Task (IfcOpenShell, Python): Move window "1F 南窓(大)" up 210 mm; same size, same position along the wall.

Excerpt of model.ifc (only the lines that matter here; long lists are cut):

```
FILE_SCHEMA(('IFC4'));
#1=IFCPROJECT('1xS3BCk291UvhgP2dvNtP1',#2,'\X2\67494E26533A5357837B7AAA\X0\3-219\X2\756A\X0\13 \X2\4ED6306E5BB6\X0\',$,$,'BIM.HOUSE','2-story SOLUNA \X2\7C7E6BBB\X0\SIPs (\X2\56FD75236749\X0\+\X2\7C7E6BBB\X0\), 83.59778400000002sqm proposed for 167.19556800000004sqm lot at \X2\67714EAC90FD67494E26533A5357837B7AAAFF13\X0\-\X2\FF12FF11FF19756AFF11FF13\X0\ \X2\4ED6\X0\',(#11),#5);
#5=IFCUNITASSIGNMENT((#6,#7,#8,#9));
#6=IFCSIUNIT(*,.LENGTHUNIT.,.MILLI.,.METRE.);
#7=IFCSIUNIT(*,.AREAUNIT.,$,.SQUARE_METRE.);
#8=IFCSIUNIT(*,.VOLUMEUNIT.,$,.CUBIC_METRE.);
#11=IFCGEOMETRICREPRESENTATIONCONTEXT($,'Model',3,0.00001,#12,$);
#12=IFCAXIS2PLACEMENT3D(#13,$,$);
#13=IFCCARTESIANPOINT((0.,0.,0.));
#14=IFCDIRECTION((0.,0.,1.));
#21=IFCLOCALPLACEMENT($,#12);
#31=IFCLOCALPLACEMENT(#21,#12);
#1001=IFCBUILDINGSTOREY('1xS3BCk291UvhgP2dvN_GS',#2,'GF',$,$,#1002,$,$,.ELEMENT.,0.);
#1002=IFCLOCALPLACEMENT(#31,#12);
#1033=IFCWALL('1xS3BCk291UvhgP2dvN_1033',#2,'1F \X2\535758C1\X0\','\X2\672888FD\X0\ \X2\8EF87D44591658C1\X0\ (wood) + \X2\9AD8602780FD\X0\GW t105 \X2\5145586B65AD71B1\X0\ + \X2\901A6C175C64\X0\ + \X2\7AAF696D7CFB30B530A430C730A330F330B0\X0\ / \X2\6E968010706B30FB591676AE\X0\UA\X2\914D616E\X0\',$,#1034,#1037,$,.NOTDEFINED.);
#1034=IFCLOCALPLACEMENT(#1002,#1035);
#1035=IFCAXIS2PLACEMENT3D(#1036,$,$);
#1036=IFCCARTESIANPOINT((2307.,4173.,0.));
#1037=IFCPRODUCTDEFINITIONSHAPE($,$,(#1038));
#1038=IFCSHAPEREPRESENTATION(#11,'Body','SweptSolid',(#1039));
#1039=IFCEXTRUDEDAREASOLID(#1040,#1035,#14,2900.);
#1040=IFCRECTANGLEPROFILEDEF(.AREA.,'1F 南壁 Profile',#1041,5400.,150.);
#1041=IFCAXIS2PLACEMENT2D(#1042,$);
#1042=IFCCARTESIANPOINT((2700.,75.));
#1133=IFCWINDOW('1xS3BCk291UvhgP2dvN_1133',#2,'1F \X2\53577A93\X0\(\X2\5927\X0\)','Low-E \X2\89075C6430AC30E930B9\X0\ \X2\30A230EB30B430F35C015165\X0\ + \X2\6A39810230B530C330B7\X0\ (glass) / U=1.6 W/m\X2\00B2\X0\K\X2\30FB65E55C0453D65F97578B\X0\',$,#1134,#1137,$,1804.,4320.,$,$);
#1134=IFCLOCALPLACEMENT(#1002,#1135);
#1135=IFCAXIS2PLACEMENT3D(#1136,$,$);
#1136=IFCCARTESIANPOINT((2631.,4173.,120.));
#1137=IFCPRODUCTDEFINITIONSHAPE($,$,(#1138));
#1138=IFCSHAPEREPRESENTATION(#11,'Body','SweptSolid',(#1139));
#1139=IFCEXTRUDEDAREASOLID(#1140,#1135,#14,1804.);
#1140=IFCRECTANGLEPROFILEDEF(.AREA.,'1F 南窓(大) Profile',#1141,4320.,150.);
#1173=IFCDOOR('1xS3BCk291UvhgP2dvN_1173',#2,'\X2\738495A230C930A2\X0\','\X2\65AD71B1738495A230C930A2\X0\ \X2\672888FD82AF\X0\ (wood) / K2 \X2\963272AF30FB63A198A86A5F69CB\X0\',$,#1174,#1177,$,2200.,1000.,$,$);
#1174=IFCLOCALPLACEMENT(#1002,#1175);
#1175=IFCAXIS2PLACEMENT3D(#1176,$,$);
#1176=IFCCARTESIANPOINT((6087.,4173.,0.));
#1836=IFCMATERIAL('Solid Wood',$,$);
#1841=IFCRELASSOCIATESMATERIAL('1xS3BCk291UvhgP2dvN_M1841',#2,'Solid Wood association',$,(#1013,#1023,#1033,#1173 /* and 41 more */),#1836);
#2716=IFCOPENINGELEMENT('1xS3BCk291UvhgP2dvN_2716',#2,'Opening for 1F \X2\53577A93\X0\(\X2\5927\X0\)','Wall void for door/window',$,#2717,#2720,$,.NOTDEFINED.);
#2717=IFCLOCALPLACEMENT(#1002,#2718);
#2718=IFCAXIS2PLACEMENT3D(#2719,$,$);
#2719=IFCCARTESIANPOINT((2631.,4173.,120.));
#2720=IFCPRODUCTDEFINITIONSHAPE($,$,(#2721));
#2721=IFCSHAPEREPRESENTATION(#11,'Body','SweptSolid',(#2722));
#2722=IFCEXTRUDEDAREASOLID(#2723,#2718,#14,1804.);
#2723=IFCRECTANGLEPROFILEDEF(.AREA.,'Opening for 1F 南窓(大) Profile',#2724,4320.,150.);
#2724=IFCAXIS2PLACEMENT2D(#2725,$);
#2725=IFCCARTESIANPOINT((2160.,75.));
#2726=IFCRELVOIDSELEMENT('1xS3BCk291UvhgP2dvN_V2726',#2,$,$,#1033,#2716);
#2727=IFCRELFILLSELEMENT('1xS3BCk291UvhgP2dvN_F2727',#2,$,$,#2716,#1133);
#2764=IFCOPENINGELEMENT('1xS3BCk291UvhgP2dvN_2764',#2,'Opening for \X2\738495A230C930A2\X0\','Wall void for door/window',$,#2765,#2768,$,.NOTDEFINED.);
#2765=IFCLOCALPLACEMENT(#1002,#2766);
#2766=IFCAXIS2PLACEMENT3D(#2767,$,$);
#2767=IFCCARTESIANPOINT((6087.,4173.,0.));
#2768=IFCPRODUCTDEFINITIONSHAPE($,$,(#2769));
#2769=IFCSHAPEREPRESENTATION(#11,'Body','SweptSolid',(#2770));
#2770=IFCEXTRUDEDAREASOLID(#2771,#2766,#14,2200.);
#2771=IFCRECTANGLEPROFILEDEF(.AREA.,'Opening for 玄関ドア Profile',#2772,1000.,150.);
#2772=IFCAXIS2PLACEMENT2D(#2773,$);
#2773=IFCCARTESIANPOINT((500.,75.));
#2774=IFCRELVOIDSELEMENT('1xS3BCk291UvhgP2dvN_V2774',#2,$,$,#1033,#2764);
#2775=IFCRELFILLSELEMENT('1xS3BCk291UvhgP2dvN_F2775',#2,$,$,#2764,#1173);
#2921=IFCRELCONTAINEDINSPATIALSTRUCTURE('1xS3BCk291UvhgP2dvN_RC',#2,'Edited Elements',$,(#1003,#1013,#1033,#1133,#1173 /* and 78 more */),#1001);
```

```python
import numpy as np
import ifcopenshell
import ifcopenshell.api.geometry
import ifcopenshell.util.placement
import ifcopenshell.util.unit

model = ifcopenshell.open("model.ifc")
unit_scale = ifcopenshell.util.unit.calculate_unit_scale(model)

window = model.by_guid("1xS3BCk291UvhgP2dvN_1133")
opening = window.FillsVoids[0].RelatingOpeningElement
dz = 210.0

shift = np.array([0.0, 0.0, dz])
# The window is not placed relative to its opening, so move both.
for product in (opening, window):
    matrix = ifcopenshell.util.placement.get_local_placement(product.ObjectPlacement)
    matrix[:3, 3] += shift
    ifcopenshell.api.geometry.edit_object_placement(model, product=product, matrix=matrix, is_si=False)

print(f"moved by {dz * unit_scale:+.3f} m")

model.write("model_v2.ifc")
```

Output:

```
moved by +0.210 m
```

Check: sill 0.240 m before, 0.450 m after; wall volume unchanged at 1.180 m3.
